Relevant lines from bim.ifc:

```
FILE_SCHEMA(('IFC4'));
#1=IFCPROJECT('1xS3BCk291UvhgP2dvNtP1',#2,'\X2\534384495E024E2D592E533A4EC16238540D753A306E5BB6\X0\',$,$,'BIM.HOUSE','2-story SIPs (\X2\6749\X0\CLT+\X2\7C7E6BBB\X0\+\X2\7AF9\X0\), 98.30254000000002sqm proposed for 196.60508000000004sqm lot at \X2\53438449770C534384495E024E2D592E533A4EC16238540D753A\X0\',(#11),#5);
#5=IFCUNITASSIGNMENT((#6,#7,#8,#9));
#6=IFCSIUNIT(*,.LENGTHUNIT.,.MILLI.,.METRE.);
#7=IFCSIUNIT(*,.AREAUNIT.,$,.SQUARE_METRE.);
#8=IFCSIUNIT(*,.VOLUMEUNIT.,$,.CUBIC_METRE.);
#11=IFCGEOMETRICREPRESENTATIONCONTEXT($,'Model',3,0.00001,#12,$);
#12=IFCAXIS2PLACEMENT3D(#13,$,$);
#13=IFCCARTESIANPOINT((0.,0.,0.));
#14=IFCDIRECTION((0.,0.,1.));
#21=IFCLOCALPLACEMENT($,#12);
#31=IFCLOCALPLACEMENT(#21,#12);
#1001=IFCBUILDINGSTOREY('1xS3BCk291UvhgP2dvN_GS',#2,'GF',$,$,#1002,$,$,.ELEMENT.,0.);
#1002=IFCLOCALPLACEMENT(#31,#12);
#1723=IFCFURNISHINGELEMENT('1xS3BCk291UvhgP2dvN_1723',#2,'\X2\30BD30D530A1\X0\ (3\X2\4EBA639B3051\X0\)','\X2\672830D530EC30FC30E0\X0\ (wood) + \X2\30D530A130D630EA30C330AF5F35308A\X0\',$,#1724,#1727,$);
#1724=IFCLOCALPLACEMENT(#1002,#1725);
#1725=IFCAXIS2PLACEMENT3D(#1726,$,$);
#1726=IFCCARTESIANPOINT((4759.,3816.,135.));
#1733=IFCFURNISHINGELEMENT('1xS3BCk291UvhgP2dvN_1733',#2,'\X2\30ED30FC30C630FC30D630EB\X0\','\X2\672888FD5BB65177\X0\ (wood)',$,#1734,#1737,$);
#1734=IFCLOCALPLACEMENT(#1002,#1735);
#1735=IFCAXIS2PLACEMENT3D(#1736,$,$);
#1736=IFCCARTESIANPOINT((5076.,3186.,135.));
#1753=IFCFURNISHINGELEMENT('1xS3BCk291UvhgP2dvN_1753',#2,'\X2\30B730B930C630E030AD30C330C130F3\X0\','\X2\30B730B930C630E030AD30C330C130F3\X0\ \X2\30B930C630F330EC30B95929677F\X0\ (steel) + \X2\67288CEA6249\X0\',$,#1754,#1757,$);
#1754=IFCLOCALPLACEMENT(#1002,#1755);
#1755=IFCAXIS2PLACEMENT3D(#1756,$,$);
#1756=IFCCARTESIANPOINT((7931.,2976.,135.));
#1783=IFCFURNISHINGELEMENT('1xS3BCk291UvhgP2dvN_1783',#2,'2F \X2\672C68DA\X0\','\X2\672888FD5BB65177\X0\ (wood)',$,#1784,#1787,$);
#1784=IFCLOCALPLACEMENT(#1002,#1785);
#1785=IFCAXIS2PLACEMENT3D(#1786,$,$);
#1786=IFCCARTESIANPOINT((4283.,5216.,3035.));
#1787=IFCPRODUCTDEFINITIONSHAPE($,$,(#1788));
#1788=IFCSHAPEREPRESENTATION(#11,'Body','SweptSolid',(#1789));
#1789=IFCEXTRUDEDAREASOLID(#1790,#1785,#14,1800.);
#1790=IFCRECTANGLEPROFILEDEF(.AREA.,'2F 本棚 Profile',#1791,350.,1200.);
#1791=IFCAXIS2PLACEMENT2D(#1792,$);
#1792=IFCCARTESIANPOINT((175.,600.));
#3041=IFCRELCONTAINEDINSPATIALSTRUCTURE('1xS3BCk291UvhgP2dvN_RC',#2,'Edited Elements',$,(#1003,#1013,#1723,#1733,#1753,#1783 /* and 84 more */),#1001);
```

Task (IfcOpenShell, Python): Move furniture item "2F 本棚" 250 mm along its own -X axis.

```python
import ifcopenshell
import ifcopenshell.api.geometry
import ifcopenshell.util.placement

model = ifcopenshell.open("bim.ifc")

item = model.by_guid("1xS3BCk291UvhgP2dvN_1783")
matrix = ifcopenshell.util.placement.get_local_placement(item.ObjectPlacement)
matrix[:3, 3] -= matrix[:3, 0] * 250.0
ifcopenshell.api.geometry.edit_object_placement(model, product=item, matrix=matrix, is_si=False)

print(ifcopenshell.util.placement.get_local_placement(item.ObjectPlacement).round(3) + 0.0)

model.write("bim_rev.ifc")
```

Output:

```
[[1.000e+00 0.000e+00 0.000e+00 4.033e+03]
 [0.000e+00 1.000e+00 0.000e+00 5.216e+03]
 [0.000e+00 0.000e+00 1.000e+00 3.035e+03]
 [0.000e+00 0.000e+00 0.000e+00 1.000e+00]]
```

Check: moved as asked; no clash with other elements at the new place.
